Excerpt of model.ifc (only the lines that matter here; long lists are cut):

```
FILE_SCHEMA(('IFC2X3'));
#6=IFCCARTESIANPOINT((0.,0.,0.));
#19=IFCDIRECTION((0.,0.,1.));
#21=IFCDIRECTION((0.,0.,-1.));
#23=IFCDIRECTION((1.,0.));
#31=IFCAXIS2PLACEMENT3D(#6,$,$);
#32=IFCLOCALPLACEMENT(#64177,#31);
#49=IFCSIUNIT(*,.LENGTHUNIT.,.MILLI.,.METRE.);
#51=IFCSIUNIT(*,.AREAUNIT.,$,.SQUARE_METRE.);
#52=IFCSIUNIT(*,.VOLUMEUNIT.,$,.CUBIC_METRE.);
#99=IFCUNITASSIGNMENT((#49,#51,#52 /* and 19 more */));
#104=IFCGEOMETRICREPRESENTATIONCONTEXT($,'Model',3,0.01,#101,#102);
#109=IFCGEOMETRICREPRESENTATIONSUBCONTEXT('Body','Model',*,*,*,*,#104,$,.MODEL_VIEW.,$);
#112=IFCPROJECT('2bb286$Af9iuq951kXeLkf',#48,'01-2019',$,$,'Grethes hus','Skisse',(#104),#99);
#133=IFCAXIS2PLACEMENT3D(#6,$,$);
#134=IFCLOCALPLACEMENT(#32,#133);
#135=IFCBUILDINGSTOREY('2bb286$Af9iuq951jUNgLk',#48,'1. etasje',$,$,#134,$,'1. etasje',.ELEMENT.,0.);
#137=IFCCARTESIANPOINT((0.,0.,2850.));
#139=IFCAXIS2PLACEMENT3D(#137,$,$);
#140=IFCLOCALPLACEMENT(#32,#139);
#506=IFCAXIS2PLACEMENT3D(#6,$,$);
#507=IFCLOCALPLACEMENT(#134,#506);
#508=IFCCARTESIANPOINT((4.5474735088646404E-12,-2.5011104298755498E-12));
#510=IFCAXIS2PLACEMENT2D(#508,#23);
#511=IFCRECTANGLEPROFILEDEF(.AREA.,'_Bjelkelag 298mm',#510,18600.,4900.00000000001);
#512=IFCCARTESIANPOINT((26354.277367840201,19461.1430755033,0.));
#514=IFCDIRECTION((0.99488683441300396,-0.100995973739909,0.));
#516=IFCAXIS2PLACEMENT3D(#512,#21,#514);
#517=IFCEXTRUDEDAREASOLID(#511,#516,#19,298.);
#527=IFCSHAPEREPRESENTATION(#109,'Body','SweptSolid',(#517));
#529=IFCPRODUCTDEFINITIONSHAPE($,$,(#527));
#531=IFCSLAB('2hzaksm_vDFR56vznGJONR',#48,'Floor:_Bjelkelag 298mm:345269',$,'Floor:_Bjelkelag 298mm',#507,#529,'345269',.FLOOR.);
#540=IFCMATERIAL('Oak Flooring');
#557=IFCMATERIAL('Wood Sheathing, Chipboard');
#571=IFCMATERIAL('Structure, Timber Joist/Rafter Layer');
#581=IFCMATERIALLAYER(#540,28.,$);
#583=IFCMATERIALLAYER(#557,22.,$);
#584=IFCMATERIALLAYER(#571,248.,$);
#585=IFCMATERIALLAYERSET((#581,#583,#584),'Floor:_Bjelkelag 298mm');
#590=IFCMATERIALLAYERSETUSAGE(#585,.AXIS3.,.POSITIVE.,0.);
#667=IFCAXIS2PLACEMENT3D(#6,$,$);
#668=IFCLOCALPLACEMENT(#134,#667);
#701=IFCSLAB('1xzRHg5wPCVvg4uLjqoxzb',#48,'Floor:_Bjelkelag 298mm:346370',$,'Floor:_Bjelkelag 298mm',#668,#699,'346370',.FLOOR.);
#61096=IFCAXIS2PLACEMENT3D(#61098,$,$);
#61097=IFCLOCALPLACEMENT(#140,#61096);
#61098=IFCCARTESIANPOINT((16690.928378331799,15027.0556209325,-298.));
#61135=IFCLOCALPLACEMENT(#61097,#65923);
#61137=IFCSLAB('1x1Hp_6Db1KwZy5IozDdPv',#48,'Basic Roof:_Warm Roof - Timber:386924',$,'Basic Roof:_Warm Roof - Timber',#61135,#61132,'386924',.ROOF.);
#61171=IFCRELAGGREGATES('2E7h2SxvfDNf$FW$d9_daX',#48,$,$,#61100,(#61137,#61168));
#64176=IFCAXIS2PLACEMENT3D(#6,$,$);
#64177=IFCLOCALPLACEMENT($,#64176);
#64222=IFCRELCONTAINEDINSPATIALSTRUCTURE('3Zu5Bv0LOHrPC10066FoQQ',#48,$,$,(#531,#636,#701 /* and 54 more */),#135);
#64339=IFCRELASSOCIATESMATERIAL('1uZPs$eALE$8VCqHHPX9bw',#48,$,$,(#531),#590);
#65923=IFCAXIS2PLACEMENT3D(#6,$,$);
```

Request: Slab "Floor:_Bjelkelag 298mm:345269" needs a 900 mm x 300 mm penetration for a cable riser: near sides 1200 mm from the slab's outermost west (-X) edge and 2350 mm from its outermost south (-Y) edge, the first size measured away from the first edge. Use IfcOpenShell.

```python
import numpy as np
import ifcopenshell
import ifcopenshell.api.feature
import ifcopenshell.api.geometry
import ifcopenshell.api.root
import ifcopenshell.geom
import ifcopenshell.util.placement
import ifcopenshell.util.representation
import ifcopenshell.util.shape
import ifcopenshell.util.unit

model = ifcopenshell.open("model.ifc")
unit_scale = ifcopenshell.util.unit.calculate_unit_scale(model)
settings = ifcopenshell.geom.settings()


def volume(element):
    """Net volume in cubic metres, openings subtracted."""
    shape = ifcopenshell.geom.create_shape(settings, element)
    return ifcopenshell.util.shape.get_volume(shape.geometry)


slab = model.by_guid("2hzaksm_vDFR56vznGJONR")
before = volume(slab)

# Extent in the slab's own axes, in metres. The edges named are its -X and -Y sides.
slab_shape = ifcopenshell.geom.create_shape(settings, slab)
vertices = ifcopenshell.util.shape.get_vertices(slab_shape.geometry)
x_min, y_min, bottom = vertices.min(axis=0)
top = vertices[:, 2].max()

opening = ifcopenshell.api.root.create_entity(model, ifc_class="IfcOpeningElement", name="Cable riser opening")
context = ifcopenshell.util.representation.get_context(model, "Model", "Body", "MODEL_VIEW")
width, depth = 0.9, 0.3
outline = [(0.0, 0.0), (width, 0.0), (width, depth), (0.0, depth), (0.0, 0.0)]
# Overshoot both faces by 50 mm so the cut is clean.
shape = ifcopenshell.api.geometry.add_slab_representation(
    model, context=context, depth=top - bottom + 0.1, polyline=outline
)
ifcopenshell.api.geometry.assign_representation(model, product=opening, representation=shape)

matrix = ifcopenshell.util.placement.get_local_placement(slab.ObjectPlacement)
matrix[:, 3] = matrix @ np.append(np.array([x_min + 1.2, y_min + 2.35, bottom - 0.05]) / unit_scale, 1.0)
ifcopenshell.api.geometry.edit_object_placement(model, product=opening, matrix=matrix, is_si=False)
ifcopenshell.api.feature.add_feature(model, feature=opening, element=slab)

after = volume(slab)

print(f"slab volume {before:.3f} -> {after:.3f} m3")

model.write("model_updated.ifc")
```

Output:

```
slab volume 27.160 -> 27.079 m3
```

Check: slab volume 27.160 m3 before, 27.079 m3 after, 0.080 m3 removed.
